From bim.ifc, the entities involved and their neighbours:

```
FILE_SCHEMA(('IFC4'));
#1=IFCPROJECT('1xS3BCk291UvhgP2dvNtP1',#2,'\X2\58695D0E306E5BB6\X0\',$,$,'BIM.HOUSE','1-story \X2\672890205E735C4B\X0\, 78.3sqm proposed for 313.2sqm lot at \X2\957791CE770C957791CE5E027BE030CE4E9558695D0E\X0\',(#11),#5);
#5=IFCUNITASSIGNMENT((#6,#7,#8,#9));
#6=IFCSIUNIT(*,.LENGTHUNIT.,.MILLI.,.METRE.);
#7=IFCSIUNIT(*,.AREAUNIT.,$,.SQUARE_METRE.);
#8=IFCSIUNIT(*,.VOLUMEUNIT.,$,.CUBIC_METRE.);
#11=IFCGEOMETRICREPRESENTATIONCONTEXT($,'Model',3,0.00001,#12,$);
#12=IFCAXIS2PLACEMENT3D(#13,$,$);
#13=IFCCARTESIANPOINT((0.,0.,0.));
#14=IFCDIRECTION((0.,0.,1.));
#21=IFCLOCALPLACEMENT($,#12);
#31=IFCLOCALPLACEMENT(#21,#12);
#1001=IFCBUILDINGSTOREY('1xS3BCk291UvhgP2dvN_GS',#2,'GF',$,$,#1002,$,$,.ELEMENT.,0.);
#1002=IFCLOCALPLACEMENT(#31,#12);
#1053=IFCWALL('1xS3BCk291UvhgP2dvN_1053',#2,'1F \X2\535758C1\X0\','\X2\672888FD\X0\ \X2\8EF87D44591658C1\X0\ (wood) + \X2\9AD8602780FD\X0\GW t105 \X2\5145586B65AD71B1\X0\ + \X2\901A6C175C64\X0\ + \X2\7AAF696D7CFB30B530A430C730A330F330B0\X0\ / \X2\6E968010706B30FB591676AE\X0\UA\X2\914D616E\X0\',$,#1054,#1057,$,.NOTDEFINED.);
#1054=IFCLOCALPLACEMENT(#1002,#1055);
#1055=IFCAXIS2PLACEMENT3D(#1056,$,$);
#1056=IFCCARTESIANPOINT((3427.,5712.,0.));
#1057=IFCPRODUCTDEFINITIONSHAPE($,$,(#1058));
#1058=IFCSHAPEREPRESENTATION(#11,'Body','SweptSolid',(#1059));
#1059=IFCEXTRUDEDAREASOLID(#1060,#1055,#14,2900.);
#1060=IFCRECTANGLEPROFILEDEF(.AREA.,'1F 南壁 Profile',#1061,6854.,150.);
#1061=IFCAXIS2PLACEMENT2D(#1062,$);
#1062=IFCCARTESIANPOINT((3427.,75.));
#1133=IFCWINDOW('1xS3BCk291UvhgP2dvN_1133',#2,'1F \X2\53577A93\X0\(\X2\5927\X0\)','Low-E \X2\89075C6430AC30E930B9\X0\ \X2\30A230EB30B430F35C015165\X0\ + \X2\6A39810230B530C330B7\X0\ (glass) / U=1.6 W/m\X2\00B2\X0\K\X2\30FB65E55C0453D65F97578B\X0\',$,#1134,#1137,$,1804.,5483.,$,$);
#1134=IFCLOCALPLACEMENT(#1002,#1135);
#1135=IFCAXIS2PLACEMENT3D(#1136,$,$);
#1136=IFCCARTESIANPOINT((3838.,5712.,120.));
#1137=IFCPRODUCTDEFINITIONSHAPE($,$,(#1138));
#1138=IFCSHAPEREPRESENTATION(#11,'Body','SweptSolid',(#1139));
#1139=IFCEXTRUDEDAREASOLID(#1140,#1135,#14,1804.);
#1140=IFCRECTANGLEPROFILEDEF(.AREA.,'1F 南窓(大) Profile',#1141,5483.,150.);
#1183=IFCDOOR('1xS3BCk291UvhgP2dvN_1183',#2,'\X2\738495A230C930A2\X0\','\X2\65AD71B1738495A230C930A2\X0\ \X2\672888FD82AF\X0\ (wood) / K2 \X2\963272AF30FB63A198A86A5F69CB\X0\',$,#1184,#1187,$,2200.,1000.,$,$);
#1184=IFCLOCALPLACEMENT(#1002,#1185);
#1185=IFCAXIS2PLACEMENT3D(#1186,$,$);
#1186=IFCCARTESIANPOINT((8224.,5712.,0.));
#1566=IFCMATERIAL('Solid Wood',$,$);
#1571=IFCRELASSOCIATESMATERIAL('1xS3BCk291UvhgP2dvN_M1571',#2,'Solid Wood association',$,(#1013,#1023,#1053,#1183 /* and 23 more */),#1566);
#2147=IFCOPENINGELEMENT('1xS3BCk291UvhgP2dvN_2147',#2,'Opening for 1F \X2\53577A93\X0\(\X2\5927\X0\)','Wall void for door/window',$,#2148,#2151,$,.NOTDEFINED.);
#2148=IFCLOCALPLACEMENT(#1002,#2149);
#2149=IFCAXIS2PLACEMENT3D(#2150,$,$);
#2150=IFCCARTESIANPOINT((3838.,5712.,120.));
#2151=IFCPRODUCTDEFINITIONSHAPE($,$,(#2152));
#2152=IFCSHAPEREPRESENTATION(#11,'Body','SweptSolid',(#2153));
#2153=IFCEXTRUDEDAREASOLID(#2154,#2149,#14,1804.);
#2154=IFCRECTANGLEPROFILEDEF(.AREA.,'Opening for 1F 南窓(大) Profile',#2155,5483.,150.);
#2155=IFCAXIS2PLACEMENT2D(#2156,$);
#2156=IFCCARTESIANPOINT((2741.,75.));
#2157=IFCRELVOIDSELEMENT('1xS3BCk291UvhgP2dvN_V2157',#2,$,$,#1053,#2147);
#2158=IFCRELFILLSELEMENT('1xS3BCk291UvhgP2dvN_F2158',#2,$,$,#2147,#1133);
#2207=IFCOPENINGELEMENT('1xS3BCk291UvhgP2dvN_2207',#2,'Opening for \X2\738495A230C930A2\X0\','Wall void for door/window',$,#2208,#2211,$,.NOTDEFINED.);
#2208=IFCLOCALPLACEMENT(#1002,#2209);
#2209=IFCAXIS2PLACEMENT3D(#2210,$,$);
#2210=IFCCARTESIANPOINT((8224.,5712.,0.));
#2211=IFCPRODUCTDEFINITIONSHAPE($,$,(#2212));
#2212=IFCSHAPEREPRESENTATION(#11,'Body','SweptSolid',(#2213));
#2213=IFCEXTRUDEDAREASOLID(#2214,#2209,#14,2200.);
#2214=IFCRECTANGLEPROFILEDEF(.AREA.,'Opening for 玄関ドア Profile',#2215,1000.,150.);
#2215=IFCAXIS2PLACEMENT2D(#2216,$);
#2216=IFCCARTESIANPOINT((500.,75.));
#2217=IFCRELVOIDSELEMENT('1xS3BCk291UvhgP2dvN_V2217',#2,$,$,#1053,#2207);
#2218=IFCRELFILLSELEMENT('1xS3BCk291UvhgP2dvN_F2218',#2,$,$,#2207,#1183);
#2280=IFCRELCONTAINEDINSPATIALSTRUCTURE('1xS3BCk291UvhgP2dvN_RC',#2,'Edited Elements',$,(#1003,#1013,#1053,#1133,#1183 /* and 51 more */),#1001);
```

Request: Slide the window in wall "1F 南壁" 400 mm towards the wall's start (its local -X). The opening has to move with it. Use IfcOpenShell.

```python
import ifcopenshell
import ifcopenshell.api.geometry
import ifcopenshell.util.placement
import ifcopenshell.util.unit

model = ifcopenshell.open("bim.ifc")
unit_scale = ifcopenshell.util.unit.calculate_unit_scale(model)

window = model.by_id(1133)
opening = window.FillsVoids[0].RelatingOpeningElement
wall = opening.VoidsElements[0].RelatingBuildingElement

wall_matrix = ifcopenshell.util.placement.get_local_placement(wall.ObjectPlacement)
shift = wall_matrix[:3, 0] * -0.4 / unit_scale
before = ifcopenshell.util.placement.get_local_placement(window.ObjectPlacement)[:3, 3].copy()

# The window is not placed relative to its opening, so move both.
for product in (opening, window):
    matrix = ifcopenshell.util.placement.get_local_placement(product.ObjectPlacement)
    matrix[:3, 3] += shift
    ifcopenshell.api.geometry.edit_object_placement(model, product=product, matrix=matrix, is_si=False)

after = ifcopenshell.util.placement.get_local_placement(window.ObjectPlacement)[:3, 3]
print("window moved by", (after - before).round(3) + 0.0)

model.write("bim_updated.ifc")
```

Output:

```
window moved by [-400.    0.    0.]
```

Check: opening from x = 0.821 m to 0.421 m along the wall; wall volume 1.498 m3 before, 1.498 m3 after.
